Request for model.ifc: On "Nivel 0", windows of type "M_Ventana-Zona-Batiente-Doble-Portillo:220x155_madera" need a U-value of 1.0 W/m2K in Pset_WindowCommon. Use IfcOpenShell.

First a look at what the model holds.

```python
import ifcopenshell
import ifcopenshell.util.element

model = ifcopenshell.open("model.ifc")
print(model.schema)
storey = next(s for s in model.by_type("IfcBuildingStorey") if s.Name == "Nivel 0")
windows = [e for e in ifcopenshell.util.element.get_decomposition(storey) if e.is_a("IfcWindow")]
seen = {}
for e in windows:
    element_type = ifcopenshell.util.element.get_type(e)
    key = (element_type.Name if element_type != e and element_type else None, ifcopenshell.util.element.get_pset(e, "Pset_WindowCommon", "ThermalTransmittance"))
    seen[key] = seen.get(key, 0) + 1
for (name, value), count in sorted(seen.items(), key=str):
    print(count, "x", name, "|", value)
```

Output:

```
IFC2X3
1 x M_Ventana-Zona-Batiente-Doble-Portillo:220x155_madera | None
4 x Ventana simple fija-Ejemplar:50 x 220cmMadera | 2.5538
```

```python
import ifcopenshell
import ifcopenshell.api.pset
import ifcopenshell.util.element

model = ifcopenshell.open("model.ifc")

storey = next(s for s in model.by_type("IfcBuildingStorey") if s.Name == "Nivel 0")
windows = [e for e in ifcopenshell.util.element.get_decomposition(storey) if e.is_a("IfcWindow")]

count = 0
for e in windows:
    element_type = ifcopenshell.util.element.get_type(e)
    if element_type in (None, e) or element_type.Name != "M_Ventana-Zona-Batiente-Doble-Portillo:220x155_madera":
        continue
    # add_pset returns the element's existing set when there is one.
    pset = ifcopenshell.api.pset.add_pset(model, product=e, name="Pset_WindowCommon")
    ifcopenshell.api.pset.edit_pset(model, pset=pset, properties={"ThermalTransmittance": 1.0})
    count += 1

print(count, "windows updated")

model.write("model_edited.ifc")
```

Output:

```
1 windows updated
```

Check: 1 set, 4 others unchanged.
